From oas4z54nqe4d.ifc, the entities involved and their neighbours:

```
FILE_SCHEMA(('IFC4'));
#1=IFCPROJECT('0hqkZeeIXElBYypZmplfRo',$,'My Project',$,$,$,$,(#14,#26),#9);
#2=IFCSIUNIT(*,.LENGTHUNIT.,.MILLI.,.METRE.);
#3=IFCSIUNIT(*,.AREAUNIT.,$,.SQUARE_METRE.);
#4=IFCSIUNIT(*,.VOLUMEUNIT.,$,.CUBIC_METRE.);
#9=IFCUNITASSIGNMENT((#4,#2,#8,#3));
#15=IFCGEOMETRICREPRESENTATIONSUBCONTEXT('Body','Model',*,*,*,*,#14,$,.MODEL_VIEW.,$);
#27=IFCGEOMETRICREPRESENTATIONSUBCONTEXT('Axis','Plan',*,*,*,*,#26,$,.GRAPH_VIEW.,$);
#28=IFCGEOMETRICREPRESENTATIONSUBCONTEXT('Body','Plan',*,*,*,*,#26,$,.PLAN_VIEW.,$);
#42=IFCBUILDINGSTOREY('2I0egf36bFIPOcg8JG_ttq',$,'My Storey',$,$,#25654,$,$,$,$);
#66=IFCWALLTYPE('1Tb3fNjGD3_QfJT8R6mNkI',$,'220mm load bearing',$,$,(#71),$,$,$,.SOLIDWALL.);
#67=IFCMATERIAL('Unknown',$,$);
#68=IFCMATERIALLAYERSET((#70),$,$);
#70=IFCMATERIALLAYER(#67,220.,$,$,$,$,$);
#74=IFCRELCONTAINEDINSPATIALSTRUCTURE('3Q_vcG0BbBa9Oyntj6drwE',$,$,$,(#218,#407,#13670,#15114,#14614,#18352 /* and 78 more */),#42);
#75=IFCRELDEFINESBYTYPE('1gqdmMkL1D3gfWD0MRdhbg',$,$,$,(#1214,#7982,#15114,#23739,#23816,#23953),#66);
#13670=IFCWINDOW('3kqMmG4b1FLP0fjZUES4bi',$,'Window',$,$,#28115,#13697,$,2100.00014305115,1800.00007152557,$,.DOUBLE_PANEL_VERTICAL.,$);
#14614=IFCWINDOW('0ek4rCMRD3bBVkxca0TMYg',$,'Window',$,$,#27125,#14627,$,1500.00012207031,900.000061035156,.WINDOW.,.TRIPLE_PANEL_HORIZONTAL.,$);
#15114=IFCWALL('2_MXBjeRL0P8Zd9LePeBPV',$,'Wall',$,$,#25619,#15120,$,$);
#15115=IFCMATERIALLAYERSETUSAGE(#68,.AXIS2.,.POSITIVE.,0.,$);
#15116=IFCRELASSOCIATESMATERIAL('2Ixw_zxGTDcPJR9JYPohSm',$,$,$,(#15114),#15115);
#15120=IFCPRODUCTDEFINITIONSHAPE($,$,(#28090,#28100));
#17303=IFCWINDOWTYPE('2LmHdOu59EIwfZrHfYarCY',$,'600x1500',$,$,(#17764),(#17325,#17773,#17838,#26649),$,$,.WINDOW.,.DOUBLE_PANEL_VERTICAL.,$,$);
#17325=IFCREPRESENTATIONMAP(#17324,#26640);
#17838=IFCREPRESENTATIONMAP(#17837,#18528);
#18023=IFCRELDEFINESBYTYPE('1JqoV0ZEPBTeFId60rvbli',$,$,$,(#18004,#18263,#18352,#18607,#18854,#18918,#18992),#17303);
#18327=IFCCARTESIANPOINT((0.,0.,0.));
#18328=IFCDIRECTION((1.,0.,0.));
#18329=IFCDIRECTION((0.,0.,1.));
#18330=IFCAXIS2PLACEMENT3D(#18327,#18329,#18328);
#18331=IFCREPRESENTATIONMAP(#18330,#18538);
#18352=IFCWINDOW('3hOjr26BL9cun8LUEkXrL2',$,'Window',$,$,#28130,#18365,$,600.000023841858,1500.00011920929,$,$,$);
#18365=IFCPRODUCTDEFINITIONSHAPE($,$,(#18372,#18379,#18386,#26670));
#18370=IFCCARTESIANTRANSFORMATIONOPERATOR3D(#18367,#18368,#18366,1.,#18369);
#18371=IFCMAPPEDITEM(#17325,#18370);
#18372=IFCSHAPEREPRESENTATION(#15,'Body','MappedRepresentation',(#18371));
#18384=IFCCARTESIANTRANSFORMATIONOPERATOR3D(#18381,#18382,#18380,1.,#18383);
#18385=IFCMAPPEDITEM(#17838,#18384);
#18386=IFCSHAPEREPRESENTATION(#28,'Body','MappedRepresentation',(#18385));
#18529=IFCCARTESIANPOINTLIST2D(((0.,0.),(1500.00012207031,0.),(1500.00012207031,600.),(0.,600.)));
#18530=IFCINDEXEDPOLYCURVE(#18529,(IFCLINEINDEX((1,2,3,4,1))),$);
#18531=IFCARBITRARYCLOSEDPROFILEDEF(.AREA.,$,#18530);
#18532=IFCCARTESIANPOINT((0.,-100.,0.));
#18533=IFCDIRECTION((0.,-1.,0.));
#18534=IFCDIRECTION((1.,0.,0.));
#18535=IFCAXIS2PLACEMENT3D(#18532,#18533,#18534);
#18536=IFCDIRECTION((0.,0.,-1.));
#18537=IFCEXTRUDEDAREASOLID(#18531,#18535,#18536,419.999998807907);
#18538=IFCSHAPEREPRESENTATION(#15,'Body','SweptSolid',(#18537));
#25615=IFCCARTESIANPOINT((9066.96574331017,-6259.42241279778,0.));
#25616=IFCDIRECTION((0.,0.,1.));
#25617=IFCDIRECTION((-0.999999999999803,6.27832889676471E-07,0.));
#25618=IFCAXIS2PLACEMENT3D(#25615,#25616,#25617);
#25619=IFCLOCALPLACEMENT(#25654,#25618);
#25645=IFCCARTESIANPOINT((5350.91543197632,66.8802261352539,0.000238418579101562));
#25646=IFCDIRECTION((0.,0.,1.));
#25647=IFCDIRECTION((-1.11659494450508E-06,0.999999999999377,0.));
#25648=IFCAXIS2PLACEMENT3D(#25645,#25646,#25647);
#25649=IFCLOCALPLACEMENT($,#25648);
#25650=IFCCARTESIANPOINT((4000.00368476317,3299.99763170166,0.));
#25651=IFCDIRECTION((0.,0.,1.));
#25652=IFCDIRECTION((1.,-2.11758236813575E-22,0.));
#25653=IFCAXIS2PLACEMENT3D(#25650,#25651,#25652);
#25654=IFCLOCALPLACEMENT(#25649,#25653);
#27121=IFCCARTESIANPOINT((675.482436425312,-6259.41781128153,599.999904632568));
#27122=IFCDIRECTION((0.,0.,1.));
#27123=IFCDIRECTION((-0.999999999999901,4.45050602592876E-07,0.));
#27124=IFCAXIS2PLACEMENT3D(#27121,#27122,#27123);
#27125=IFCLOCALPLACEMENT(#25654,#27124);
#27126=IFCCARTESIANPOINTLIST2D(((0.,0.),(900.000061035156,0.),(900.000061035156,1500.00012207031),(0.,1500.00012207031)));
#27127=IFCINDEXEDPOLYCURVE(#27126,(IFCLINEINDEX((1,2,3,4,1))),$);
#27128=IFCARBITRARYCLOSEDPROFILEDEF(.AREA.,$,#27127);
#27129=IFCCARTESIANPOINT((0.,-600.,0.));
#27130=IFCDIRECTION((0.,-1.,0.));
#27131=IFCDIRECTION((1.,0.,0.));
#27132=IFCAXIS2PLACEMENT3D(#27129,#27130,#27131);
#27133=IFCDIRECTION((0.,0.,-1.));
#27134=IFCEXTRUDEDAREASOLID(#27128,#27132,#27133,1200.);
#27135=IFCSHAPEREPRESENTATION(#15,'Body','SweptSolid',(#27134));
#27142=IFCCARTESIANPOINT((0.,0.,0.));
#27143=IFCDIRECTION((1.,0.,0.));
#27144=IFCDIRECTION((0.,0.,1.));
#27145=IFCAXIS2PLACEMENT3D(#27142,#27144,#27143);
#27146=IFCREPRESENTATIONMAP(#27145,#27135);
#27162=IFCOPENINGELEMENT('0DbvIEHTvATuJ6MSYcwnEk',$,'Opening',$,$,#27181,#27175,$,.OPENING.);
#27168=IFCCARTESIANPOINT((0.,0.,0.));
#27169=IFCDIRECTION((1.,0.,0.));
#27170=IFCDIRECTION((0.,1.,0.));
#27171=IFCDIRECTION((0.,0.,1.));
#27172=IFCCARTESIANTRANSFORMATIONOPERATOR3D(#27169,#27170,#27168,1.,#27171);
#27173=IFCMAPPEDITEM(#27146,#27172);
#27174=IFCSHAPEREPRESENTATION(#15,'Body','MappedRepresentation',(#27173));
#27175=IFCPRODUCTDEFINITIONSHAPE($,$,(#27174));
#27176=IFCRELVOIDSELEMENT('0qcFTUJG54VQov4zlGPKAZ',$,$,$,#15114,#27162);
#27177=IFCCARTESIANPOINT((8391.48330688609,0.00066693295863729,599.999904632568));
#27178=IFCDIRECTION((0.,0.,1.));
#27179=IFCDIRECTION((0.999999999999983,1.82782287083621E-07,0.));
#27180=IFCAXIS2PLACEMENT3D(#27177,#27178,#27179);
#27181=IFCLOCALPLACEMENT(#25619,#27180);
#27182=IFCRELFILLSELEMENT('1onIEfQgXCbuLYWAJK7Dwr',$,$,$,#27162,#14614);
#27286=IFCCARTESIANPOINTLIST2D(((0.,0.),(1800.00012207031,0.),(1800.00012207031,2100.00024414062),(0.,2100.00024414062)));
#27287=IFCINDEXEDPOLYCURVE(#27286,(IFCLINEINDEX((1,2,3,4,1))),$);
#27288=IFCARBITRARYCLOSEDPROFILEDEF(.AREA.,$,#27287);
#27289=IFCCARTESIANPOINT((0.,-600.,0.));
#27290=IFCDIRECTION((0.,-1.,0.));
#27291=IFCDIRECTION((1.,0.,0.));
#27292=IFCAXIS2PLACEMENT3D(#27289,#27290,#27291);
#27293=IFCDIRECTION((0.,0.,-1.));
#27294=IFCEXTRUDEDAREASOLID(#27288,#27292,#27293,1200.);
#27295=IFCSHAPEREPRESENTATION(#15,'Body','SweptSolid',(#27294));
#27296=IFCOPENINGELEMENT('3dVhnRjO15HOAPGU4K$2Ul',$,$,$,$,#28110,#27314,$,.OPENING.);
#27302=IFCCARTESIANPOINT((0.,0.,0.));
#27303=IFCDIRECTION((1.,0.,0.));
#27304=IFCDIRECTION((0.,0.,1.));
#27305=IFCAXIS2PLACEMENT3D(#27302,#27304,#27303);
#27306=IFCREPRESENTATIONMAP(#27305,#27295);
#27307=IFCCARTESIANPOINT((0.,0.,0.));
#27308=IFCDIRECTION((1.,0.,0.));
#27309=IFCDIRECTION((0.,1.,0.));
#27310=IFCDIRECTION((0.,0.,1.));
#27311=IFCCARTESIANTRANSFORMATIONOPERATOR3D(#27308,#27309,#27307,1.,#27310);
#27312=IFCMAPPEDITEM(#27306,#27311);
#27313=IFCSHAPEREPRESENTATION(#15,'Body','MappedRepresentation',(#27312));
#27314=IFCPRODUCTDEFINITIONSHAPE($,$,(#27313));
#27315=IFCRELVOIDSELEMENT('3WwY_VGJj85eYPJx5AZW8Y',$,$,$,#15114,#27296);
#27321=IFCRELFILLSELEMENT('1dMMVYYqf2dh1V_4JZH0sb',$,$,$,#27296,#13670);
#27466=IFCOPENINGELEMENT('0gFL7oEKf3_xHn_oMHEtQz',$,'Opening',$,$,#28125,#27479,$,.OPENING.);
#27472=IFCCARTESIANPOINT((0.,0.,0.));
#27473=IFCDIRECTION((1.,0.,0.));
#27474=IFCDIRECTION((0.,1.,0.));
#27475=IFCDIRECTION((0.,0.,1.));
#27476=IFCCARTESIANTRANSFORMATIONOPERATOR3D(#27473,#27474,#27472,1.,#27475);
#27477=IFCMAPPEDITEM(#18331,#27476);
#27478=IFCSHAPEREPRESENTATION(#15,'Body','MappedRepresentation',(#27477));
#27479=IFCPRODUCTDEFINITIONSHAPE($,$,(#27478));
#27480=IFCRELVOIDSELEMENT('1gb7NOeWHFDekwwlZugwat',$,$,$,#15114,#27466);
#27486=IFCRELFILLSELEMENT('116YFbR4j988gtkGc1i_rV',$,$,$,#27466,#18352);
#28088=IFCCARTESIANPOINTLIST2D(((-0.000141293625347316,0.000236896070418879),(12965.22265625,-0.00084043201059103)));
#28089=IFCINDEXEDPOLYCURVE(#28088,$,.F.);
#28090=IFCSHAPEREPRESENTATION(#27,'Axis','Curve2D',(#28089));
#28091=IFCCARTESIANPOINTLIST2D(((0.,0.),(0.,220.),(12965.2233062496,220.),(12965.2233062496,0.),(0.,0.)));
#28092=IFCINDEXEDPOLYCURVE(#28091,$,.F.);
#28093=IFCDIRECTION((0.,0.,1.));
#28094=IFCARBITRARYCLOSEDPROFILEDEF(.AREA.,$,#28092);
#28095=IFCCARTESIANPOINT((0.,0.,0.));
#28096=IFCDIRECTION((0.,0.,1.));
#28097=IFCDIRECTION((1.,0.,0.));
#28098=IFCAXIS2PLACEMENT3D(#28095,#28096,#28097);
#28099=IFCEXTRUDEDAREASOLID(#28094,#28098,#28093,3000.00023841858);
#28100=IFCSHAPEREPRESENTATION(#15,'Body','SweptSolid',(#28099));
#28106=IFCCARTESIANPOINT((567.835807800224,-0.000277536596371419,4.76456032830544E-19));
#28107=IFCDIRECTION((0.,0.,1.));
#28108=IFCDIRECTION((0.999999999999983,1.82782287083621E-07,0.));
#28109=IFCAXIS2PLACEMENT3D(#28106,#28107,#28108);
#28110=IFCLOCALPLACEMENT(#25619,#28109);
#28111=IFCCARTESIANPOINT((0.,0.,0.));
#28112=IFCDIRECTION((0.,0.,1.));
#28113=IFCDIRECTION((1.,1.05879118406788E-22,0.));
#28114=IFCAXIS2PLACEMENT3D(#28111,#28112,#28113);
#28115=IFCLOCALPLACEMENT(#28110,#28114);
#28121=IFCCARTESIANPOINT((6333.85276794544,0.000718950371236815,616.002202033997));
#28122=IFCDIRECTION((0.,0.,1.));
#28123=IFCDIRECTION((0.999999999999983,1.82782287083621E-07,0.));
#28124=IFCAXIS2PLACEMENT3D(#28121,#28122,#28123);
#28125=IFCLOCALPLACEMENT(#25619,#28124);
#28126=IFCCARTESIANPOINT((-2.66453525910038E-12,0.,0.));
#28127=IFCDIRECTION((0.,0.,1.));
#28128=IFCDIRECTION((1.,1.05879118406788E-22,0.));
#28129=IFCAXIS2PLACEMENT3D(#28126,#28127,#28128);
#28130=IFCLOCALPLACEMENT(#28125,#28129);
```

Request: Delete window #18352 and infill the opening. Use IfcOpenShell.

```python
import ifcopenshell
import ifcopenshell.api.feature
import ifcopenshell.api.root
import ifcopenshell.geom
import ifcopenshell.util.shape

model = ifcopenshell.open("oas4z54nqe4d.ifc")
settings = ifcopenshell.geom.settings()


def volume(element):
    """Net volume in cubic metres, openings subtracted."""
    shape = ifcopenshell.geom.create_shape(settings, element)
    return ifcopenshell.util.shape.get_volume(shape.geometry)


window = model.by_guid("3hOjr26BL9cun8LUEkXrL2")
opening = window.FillsVoids[0].RelatingOpeningElement
wall = opening.VoidsElements[0].RelatingBuildingElement
before = volume(wall)

ifcopenshell.api.root.remove_product(model, product=window)
ifcopenshell.api.feature.remove_feature(model, feature=opening)

after = volume(wall)

print(f"wall volume {before:.3f} -> {after:.3f} m3")

model.write("oas4z54nqe4d_v2.ifc")
```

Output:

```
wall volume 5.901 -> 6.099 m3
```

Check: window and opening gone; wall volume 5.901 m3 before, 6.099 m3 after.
